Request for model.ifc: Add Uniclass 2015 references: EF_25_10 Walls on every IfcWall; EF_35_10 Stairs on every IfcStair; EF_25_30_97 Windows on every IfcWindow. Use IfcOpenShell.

First a look at what the model holds.

```python
import ifcopenshell

model = ifcopenshell.open("model.ifc")
print(model.schema)
print("classifications:", [c.Name for c in model.by_type("IfcClassification")])
for ifc_class in ("IfcDoor", "IfcRoof", "IfcStair", "IfcWall", "IfcWindow"):
    print(ifc_class, len(model.by_type(ifc_class)))
```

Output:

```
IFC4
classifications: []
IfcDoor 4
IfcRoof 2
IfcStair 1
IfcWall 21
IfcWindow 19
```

```python
import ifcopenshell
import ifcopenshell.api.classification

model = ifcopenshell.open("model.ifc")

system = ifcopenshell.api.classification.add_classification(model, classification="Uniclass 2015")

codes = {
    "IfcWall": ("EF_25_10", "Walls"),
    "IfcStair": ("EF_35_10", "Stairs"),
    "IfcWindow": ("EF_25_30_97", "Windows"),
}
for ifc_class, (code, name) in codes.items():
    products = model.by_type(ifc_class)
    ifcopenshell.api.classification.add_reference(
        model, products=products, classification=system, identification=code, name=name
    )
    print(code, len(products))

model.write("model-out.ifc")
```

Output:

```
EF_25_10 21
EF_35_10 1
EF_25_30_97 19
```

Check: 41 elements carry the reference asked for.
